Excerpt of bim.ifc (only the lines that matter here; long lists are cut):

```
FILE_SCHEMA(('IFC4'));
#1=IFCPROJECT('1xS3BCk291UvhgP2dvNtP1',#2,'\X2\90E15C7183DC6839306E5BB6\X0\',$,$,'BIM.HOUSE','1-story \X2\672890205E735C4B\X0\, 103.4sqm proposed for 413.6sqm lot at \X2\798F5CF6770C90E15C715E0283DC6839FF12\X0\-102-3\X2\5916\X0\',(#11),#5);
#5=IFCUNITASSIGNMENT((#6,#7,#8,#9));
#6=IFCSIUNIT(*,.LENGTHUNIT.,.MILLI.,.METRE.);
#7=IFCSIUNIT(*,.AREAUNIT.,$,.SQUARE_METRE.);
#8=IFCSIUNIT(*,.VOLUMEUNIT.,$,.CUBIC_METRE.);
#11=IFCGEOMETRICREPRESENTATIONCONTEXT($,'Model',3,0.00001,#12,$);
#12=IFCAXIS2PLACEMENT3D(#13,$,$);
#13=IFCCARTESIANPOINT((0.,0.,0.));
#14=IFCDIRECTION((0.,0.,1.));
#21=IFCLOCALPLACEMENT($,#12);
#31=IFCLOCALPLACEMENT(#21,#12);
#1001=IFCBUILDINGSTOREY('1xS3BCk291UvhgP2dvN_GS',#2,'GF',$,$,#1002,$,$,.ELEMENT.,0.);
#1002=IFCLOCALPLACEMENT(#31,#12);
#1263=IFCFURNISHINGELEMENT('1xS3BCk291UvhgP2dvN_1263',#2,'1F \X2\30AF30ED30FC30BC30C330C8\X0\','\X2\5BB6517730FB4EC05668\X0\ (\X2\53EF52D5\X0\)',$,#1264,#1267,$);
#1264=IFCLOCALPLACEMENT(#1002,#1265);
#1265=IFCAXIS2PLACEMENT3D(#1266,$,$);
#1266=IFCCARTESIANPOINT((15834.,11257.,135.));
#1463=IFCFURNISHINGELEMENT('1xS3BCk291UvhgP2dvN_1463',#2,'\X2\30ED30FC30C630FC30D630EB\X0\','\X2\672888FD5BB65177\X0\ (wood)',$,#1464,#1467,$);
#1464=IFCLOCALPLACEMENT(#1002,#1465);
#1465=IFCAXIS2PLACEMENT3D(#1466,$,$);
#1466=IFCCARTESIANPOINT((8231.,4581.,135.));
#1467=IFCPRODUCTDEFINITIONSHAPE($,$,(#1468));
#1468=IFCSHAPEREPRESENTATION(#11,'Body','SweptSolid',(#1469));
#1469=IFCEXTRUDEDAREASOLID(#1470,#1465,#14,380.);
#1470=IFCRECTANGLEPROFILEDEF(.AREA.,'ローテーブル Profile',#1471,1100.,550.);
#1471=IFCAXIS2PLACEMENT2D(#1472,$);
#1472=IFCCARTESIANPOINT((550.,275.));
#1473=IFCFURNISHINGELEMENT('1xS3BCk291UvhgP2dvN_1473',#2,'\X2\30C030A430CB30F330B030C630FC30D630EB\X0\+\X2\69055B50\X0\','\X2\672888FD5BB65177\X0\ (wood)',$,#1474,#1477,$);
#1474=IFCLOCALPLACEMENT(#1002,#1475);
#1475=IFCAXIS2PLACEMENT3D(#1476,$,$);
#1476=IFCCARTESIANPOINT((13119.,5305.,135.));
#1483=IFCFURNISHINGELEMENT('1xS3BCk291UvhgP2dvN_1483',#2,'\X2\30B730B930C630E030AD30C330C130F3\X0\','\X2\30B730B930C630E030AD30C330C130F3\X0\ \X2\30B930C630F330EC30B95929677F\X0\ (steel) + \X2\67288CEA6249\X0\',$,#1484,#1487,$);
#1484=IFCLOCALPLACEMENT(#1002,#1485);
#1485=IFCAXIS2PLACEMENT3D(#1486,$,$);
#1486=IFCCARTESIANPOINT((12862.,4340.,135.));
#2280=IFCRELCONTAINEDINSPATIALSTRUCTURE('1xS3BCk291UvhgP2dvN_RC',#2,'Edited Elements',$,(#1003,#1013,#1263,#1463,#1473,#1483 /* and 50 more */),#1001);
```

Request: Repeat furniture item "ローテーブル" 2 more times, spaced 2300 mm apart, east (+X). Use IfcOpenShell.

```python
import numpy as np
import ifcopenshell
import ifcopenshell.api.geometry
import ifcopenshell.api.root
import ifcopenshell.util.element
import ifcopenshell.util.placement

model = ifcopenshell.open("bim.ifc")


def reuse_history(source, copy):
    """copy_class also copies each property set's owner history, people and application; keep the originals."""
    for rel in copy.IsDefinedBy:
        if rel.is_a("IfcRelDefinesByProperties") and (history := rel.RelatingPropertyDefinition.OwnerHistory):
            rel.RelatingPropertyDefinition.OwnerHistory = source.OwnerHistory
            ifcopenshell.util.element.remove_deep2(model, history)


source = model.by_guid("1xS3BCk291UvhgP2dvN_1463")
base = ifcopenshell.util.placement.get_local_placement(source.ObjectPlacement)
step = np.array([1.0, 0.0, 0.0]) * 2300.0

for i in range(1, 3):
    copy = ifcopenshell.api.root.copy_class(model, product=source)
    copy.Representation = ifcopenshell.util.element.copy_deep(
        model, source.Representation, exclude=["IfcGeometricRepresentationContext", "IfcRepresentationMap"]
    )
    reuse_history(source, copy)
    matrix = base.copy()
    matrix[:3, 3] += i * step
    print("added at", matrix[:3, 3].round(3) + 0.0)
    ifcopenshell.api.geometry.edit_object_placement(model, product=copy, matrix=matrix, is_si=False)

model.write("bim_rev.ifc")
```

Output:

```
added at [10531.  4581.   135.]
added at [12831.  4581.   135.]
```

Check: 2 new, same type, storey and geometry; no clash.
